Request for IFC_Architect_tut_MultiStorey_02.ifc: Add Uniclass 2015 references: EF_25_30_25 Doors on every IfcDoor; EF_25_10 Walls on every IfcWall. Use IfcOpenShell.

First a look at what the model holds.

```python
import ifcopenshell

model = ifcopenshell.open("IFC_Architect_tut_MultiStorey_02.ifc")
print(model.schema)
print("classifications:", [c.Name for c in model.by_type("IfcClassification")])
for ifc_class in ("IfcDoor", "IfcRoof", "IfcStair", "IfcWall", "IfcWindow"):
    print(ifc_class, len(model.by_type(ifc_class)))
```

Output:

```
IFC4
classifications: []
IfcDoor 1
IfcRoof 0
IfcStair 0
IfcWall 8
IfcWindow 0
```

```python
import ifcopenshell
import ifcopenshell.api.classification

model = ifcopenshell.open("IFC_Architect_tut_MultiStorey_02.ifc")

system = ifcopenshell.api.classification.add_classification(model, classification="Uniclass 2015")

codes = {
    "IfcDoor": ("EF_25_30_25", "Doors"),
    "IfcWall": ("EF_25_10", "Walls"),
}
for ifc_class, (code, name) in codes.items():
    products = model.by_type(ifc_class)
    ifcopenshell.api.classification.add_reference(
        model, products=products, classification=system, identification=code, name=name
    )
    print(code, len(products))

model.write("IFC_Architect_tut_MultiStorey_02_updated.ifc")
```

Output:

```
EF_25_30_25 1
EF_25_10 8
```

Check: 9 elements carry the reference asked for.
